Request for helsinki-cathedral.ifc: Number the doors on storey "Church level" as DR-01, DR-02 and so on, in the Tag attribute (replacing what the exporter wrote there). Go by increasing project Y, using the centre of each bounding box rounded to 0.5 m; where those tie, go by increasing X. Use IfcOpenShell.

First a look at what the model holds.

```python
import ifcopenshell
import ifcopenshell.util.element
import ifcopenshell.util.placement

model = ifcopenshell.open("helsinki-cathedral.ifc")
print(model.schema)
storey = next(s for s in model.by_type("IfcBuildingStorey") if s.Name == "Church level")
doors = [e for e in ifcopenshell.util.element.get_decomposition(storey) if e.is_a("IfcDoor")]
for e in sorted(doors, key=lambda e: e.id()):
    origin = ifcopenshell.util.placement.get_local_placement(e.ObjectPlacement)[:3, 3]
    print(e.id(), e.Tag, e.Name, origin.round(2) + 0.0, sep=" | ")
```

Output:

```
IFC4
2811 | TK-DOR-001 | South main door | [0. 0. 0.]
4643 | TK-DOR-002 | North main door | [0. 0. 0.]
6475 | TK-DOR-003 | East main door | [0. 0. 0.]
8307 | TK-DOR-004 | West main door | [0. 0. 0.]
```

```python
import ifcopenshell
import ifcopenshell.geom
import ifcopenshell.util.element
import ifcopenshell.util.shape

model = ifcopenshell.open("helsinki-cathedral.ifc")
settings = ifcopenshell.geom.settings()
settings.set("use-world-coords", True)


def centre(element):
    shape = ifcopenshell.geom.create_shape(settings, element)
    return ifcopenshell.util.shape.get_bbox_centroid(shape.geometry)


storey = next(s for s in model.by_type("IfcBuildingStorey") if s.Name == "Church level")
doors = [e for e in ifcopenshell.util.element.get_decomposition(storey) if e.is_a("IfcDoor")]

# Insertion points can sit at a corner or the storey origin, so sort by the geometry (in metres).
centres = {e: centre(e) for e in doors}
doors.sort(key=lambda e: (round(centres[e][1] / 0.5), centres[e][0]))

for i, e in enumerate(doors, start=1):
    number = f"DR-{i:02d}"
    e.Tag = number
    print(e.id(), number)

model.write("helsinki-cathedral_v2.ifc")
```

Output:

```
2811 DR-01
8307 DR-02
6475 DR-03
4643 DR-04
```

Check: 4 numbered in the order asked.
